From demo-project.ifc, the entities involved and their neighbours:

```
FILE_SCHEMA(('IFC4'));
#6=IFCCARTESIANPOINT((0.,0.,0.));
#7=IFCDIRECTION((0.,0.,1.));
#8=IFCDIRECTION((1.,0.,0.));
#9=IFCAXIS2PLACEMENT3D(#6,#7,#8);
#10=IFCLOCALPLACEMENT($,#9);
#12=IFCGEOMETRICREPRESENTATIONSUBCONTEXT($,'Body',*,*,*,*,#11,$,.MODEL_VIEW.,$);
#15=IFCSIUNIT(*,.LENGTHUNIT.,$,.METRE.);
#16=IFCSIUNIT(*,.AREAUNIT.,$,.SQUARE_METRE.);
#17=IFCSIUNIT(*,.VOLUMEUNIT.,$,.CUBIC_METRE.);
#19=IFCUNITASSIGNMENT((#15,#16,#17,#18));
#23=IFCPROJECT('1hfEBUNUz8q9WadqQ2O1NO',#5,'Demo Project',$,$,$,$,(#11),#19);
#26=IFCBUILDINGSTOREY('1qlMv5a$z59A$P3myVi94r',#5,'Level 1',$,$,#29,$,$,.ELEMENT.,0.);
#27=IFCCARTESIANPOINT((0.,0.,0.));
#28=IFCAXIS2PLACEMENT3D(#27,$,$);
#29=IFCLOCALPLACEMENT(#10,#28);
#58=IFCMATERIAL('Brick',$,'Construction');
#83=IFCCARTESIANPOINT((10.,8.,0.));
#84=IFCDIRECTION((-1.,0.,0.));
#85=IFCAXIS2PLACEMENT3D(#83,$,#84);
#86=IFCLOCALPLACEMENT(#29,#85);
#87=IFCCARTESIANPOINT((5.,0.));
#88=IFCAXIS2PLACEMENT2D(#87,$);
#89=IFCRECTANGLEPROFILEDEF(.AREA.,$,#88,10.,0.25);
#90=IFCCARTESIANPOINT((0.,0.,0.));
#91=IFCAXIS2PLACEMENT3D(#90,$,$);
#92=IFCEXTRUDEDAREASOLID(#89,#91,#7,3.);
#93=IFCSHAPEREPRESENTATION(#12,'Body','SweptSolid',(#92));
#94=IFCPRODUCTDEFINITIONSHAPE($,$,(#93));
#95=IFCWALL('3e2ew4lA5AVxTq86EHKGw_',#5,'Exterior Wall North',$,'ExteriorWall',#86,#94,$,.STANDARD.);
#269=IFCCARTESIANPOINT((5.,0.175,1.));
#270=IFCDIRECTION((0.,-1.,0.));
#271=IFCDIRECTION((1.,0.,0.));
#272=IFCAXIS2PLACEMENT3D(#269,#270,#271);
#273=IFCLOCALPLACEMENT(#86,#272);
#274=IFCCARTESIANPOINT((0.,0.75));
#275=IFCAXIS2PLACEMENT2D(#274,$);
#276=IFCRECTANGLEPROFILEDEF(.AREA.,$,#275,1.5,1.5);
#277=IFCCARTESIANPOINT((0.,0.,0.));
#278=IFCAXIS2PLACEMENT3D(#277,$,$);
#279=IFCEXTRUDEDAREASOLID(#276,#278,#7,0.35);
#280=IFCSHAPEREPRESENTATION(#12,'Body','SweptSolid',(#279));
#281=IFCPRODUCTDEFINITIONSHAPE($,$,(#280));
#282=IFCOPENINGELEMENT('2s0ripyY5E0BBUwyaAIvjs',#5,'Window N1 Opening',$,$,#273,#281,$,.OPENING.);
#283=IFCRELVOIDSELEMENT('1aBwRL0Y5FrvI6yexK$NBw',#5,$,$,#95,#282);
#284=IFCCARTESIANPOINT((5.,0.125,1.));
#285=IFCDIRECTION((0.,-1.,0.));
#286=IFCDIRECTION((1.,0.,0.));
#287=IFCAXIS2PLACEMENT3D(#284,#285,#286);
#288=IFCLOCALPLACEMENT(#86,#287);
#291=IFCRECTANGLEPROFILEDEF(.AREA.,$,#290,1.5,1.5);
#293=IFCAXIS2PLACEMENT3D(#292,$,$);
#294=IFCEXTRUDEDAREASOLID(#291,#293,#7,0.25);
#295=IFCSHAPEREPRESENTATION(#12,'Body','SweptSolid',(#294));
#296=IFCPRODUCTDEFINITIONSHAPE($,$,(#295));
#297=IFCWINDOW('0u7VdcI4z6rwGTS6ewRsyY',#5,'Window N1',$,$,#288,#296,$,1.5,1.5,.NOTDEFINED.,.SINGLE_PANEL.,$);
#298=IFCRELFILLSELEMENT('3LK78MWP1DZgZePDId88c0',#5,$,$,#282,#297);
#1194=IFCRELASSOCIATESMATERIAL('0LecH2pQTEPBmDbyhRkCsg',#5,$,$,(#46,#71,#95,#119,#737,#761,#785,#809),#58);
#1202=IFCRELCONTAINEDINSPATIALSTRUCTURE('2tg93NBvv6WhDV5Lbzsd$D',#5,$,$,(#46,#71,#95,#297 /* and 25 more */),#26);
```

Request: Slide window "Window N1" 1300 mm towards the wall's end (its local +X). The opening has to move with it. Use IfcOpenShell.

```python
import ifcopenshell
import ifcopenshell.api.geometry
import ifcopenshell.util.placement
import ifcopenshell.util.unit

model = ifcopenshell.open("demo-project.ifc")
unit_scale = ifcopenshell.util.unit.calculate_unit_scale(model)

window = model.by_id(297)
opening = window.FillsVoids[0].RelatingOpeningElement
wall = opening.VoidsElements[0].RelatingBuildingElement

wall_matrix = ifcopenshell.util.placement.get_local_placement(wall.ObjectPlacement)
shift = wall_matrix[:3, 0] * 1.3 / unit_scale
before = ifcopenshell.util.placement.get_local_placement(window.ObjectPlacement)[:3, 3].copy()

# The window is not placed relative to its opening, so move both.
for product in (opening, window):
    matrix = ifcopenshell.util.placement.get_local_placement(product.ObjectPlacement)
    matrix[:3, 3] += shift
    ifcopenshell.api.geometry.edit_object_placement(model, product=product, matrix=matrix, is_si=False)

after = ifcopenshell.util.placement.get_local_placement(window.ObjectPlacement)[:3, 3]
print("window moved by", (after - before).round(3) + 0.0)

model.write("demo-project_edited.ifc")
```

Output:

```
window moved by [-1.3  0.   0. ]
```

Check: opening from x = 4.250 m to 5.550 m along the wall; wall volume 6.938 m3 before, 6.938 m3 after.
